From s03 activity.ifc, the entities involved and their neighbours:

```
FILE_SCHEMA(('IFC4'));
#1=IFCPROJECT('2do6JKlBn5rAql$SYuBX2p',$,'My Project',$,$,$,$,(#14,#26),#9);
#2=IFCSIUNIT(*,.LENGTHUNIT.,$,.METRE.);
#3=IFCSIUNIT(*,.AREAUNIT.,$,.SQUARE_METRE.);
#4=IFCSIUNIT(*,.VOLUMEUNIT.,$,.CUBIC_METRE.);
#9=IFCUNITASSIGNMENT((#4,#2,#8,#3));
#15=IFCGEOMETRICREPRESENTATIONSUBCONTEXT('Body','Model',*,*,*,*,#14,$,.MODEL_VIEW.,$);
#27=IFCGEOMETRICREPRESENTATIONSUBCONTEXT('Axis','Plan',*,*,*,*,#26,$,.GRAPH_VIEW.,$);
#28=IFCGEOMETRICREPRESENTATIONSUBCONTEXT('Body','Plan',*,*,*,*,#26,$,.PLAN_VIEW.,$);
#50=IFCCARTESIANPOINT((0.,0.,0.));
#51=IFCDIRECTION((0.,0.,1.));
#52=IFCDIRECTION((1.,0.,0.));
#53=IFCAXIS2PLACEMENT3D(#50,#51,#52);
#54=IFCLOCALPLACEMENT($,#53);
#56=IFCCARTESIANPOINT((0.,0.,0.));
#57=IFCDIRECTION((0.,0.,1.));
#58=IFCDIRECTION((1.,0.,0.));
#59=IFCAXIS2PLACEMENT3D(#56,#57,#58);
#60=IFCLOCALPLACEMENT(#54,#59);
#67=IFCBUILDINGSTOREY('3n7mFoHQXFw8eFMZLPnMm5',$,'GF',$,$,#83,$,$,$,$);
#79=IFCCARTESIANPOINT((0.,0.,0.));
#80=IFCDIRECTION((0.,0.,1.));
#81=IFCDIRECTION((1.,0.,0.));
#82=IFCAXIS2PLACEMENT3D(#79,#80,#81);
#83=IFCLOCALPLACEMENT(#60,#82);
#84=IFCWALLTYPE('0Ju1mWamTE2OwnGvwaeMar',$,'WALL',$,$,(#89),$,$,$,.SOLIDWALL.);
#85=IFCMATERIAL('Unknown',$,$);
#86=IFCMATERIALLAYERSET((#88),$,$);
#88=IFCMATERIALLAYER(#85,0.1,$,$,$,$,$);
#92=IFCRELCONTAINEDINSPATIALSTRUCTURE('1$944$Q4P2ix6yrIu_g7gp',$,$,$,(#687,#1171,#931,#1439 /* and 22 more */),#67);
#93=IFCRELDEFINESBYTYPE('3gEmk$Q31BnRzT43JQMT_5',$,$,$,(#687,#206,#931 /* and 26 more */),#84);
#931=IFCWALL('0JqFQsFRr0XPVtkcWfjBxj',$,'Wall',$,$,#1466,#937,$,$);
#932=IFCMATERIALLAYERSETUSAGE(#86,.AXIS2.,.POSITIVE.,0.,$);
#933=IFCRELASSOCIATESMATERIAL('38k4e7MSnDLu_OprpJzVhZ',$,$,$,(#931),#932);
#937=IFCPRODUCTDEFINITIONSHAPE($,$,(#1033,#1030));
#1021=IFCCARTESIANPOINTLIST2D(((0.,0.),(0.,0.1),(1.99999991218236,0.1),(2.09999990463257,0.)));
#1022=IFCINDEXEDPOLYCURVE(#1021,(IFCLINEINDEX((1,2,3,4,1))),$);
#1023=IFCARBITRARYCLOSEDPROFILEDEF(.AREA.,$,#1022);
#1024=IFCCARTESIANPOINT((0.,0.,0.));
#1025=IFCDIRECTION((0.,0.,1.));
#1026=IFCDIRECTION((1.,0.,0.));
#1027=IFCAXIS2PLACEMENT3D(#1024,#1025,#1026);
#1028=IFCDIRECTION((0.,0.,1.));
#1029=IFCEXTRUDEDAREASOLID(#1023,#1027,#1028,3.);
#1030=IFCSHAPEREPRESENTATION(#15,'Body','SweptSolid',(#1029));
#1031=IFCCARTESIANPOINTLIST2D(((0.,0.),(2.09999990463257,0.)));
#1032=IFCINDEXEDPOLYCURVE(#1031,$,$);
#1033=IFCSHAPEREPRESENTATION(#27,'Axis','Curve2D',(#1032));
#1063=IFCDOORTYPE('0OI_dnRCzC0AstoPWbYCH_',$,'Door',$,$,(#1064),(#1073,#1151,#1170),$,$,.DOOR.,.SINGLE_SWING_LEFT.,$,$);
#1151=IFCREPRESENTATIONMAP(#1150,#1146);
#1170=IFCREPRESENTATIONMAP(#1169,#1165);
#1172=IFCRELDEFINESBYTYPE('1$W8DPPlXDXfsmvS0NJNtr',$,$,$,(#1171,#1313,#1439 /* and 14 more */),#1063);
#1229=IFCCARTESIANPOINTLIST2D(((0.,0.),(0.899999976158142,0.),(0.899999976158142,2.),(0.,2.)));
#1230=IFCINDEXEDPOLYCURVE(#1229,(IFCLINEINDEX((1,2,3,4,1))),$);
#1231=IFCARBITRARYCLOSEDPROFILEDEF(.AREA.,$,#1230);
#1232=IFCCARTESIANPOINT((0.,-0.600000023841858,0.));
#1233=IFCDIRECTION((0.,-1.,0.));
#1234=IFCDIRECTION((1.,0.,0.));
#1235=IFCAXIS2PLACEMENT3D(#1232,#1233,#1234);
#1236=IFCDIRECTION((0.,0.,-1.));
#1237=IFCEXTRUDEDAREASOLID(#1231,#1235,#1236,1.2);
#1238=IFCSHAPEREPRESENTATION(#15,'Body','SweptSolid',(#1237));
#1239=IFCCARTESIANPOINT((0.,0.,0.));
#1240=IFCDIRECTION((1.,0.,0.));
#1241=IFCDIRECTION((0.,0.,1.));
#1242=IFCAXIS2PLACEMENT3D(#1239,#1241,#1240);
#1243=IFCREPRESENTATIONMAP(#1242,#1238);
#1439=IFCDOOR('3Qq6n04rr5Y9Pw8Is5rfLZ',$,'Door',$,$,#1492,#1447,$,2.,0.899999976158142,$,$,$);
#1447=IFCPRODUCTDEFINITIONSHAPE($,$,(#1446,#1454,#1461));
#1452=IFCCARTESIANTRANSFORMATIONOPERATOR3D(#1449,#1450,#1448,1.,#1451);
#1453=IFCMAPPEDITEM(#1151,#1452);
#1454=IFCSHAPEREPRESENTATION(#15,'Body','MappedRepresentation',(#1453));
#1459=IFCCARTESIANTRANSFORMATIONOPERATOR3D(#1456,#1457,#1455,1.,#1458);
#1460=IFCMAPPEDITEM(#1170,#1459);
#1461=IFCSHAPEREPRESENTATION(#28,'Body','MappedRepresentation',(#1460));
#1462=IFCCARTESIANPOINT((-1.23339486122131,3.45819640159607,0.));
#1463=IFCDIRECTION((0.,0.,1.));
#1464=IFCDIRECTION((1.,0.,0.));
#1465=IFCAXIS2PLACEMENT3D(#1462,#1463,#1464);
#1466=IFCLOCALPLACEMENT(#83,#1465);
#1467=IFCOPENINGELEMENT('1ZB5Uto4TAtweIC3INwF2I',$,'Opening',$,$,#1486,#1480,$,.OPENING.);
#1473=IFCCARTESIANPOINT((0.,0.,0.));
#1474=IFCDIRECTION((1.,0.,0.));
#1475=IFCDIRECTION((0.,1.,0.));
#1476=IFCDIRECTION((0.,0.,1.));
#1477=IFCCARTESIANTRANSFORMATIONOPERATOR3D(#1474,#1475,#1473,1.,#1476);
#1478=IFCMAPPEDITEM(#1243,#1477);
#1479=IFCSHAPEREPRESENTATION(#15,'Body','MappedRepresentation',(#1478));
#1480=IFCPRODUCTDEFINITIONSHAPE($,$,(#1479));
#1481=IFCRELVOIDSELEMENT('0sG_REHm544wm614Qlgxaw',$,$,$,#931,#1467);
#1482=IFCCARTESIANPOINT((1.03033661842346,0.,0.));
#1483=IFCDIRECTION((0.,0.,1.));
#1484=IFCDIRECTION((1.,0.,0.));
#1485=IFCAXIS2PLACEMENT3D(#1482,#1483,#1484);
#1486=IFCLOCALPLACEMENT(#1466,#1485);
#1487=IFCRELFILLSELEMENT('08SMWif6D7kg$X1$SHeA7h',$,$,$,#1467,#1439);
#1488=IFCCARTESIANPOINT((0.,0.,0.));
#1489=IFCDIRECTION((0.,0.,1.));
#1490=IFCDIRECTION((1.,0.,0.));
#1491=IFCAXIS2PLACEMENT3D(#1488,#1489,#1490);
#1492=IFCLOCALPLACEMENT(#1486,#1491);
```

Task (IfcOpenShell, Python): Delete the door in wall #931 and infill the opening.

```python
import ifcopenshell
import ifcopenshell.api.feature
import ifcopenshell.api.root
import ifcopenshell.geom
import ifcopenshell.util.shape

model = ifcopenshell.open("s03 activity.ifc")
settings = ifcopenshell.geom.settings()


def volume(element):
    """Net volume in cubic metres, openings subtracted."""
    shape = ifcopenshell.geom.create_shape(settings, element)
    return ifcopenshell.util.shape.get_volume(shape.geometry)


door = model.by_guid("3Qq6n04rr5Y9Pw8Is5rfLZ")
opening = door.FillsVoids[0].RelatingOpeningElement
wall = opening.VoidsElements[0].RelatingBuildingElement
before = volume(wall)

ifcopenshell.api.root.remove_product(model, product=door)
ifcopenshell.api.feature.remove_feature(model, feature=opening)

after = volume(wall)

print(f"wall volume {before:.3f} -> {after:.3f} m3")

model.write("s03 activity_v2.ifc")
```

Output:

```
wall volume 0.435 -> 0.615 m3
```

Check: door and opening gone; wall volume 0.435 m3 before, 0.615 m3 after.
